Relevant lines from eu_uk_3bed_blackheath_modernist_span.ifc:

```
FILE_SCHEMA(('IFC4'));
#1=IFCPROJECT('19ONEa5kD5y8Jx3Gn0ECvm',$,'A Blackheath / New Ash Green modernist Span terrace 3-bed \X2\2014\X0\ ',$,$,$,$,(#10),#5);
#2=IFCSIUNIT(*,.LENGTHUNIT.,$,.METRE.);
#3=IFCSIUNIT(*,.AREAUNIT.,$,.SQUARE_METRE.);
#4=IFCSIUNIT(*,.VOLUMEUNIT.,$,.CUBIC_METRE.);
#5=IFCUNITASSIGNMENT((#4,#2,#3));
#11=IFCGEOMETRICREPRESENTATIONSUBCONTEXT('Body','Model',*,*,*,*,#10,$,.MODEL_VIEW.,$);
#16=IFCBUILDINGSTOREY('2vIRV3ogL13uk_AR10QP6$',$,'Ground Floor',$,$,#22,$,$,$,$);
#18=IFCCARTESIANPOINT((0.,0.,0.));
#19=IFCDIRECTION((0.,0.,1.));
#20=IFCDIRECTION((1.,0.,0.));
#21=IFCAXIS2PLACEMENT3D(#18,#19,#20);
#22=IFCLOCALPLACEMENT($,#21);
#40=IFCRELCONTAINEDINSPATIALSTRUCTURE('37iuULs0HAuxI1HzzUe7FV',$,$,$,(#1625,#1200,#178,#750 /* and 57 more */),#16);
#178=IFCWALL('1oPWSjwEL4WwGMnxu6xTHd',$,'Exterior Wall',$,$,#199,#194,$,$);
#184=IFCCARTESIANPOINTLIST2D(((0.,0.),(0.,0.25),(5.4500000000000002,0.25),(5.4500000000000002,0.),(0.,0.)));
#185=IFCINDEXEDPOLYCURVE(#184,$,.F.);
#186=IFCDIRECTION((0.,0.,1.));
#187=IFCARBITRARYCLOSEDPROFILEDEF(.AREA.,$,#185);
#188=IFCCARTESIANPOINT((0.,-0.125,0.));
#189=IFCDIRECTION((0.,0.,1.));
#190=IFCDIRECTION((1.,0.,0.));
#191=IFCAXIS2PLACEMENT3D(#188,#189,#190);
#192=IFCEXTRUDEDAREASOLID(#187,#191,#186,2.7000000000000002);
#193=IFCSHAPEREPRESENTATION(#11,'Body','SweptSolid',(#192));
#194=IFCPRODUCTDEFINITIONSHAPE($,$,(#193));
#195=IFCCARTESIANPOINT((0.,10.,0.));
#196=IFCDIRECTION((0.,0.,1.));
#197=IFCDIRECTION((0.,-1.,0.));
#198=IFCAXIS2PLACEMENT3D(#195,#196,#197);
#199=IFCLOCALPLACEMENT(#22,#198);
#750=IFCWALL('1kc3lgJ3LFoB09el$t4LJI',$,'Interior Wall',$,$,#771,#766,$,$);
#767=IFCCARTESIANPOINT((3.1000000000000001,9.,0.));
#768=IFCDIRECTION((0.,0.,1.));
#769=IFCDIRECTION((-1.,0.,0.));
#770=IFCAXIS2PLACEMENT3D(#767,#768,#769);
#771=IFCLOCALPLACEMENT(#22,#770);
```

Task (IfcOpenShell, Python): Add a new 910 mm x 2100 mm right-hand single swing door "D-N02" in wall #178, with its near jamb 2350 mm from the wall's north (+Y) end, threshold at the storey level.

```python
import numpy as np
import ifcopenshell
import ifcopenshell.api.feature
import ifcopenshell.api.geometry
import ifcopenshell.api.root
import ifcopenshell.api.spatial
import ifcopenshell.geom
import ifcopenshell.util.element
import ifcopenshell.util.placement
import ifcopenshell.util.representation
import ifcopenshell.util.shape
import ifcopenshell.util.unit

model = ifcopenshell.open("eu_uk_3bed_blackheath_modernist_span.ifc")
unit_scale = ifcopenshell.util.unit.calculate_unit_scale(model)
settings = ifcopenshell.geom.settings()


def volume(element):
    """Net volume in cubic metres, openings subtracted."""
    shape = ifcopenshell.geom.create_shape(settings, element)
    return ifcopenshell.util.shape.get_volume(shape.geometry)


wall = model.by_guid("1oPWSjwEL4WwGMnxu6xTHd")
storey = ifcopenshell.util.element.get_container(wall, ifc_class="IfcBuildingStorey")
context = ifcopenshell.util.representation.get_context(model, "Model", "Body", "MODEL_VIEW")
before = volume(wall)

width, height, from_end, sill = 0.91, 2.1, 2.35, 0.0  # metres

# The wall runs along its own X axis, and the end named is its -X end.
wall_shape = ifcopenshell.geom.create_shape(settings, wall)
x, y, z = ifcopenshell.util.shape.get_vertices(wall_shape.geometry).T
start = x.min() + from_end
face, thickness = float(y.min()), float(y.max() - y.min())
wall_matrix = ifcopenshell.util.placement.get_local_placement(wall.ObjectPlacement)
level = ifcopenshell.util.placement.get_local_placement(storey.ObjectPlacement)[2, 3]


def in_wall(x, y):
    """Placement at x, y metres in the wall's axes, at sill height."""
    matrix = wall_matrix.copy()
    matrix[:, 3] = wall_matrix @ np.array([x / unit_scale, y / unit_scale, 0.0, 1.0])
    matrix[2, 3] = level + sill / unit_scale
    return matrix


# Opening: a box that overshoots both wall faces by 50 mm.
opening = ifcopenshell.api.root.create_entity(model, ifc_class="IfcOpeningElement", predefined_type="OPENING")
box = ifcopenshell.api.geometry.add_wall_representation(
    model, context=context, length=width, height=height, thickness=thickness + 0.1
)
ifcopenshell.api.geometry.assign_representation(model, product=opening, representation=box)
ifcopenshell.api.geometry.edit_object_placement(model, product=opening, matrix=in_wall(start, face - 0.05), is_si=False)
ifcopenshell.api.feature.add_feature(model, feature=opening, element=wall)

door = ifcopenshell.api.root.create_entity(model, ifc_class="IfcDoor", name="D-N02", predefined_type="DOOR")
door.OverallWidth, door.OverallHeight = width / unit_scale, height / unit_scale
door.OperationType = "SINGLE_SWING_RIGHT"
body = ifcopenshell.api.geometry.add_door_representation(
    model,
    context=context,
    overall_width=door.OverallWidth,
    overall_height=door.OverallHeight,
    operation_type="SINGLE_SWING_RIGHT",
    lining_properties={"LiningDepth": thickness / unit_scale, "ThresholdDepth": thickness / unit_scale},
)
ifcopenshell.api.geometry.assign_representation(model, product=door, representation=body)
ifcopenshell.api.spatial.assign_container(model, products=[door], relating_structure=storey)
ifcopenshell.api.feature.add_filling(model, opening=opening, element=door)

# The lining spans the wall, so the door starts at the wall face.
ifcopenshell.api.geometry.edit_object_placement(model, product=door, matrix=in_wall(start, face), is_si=False)

after = volume(wall)

print(f"wall volume {before:.3f} -> {after:.3f} m3")

model.write("eu_uk_3bed_blackheath_modernist_span_rev.ifc")
```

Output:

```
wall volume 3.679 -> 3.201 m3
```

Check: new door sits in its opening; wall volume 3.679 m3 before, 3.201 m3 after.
